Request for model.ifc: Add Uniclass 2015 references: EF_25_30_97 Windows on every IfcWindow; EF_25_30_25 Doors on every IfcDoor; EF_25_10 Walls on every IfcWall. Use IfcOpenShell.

First a look at what the model holds.

```python
import ifcopenshell

model = ifcopenshell.open("model.ifc")
print(model.schema)
print("classifications:", [c.Name for c in model.by_type("IfcClassification")])
for ifc_class in ("IfcDoor", "IfcRoof", "IfcStair", "IfcWall", "IfcWindow"):
    print(ifc_class, len(model.by_type(ifc_class)))
```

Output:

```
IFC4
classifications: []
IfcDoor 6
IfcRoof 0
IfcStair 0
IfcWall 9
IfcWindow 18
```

```python
import ifcopenshell
import ifcopenshell.api.classification

model = ifcopenshell.open("model.ifc")

system = ifcopenshell.api.classification.add_classification(model, classification="Uniclass 2015")

codes = {
    "IfcWindow": ("EF_25_30_97", "Windows"),
    "IfcDoor": ("EF_25_30_25", "Doors"),
    "IfcWall": ("EF_25_10", "Walls"),
}
for ifc_class, (code, name) in codes.items():
    products = model.by_type(ifc_class)
    ifcopenshell.api.classification.add_reference(
        model, products=products, classification=system, identification=code, name=name
    )
    print(code, len(products))

model.write("model-out.ifc")
```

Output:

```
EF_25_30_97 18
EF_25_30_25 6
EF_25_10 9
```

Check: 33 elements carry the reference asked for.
